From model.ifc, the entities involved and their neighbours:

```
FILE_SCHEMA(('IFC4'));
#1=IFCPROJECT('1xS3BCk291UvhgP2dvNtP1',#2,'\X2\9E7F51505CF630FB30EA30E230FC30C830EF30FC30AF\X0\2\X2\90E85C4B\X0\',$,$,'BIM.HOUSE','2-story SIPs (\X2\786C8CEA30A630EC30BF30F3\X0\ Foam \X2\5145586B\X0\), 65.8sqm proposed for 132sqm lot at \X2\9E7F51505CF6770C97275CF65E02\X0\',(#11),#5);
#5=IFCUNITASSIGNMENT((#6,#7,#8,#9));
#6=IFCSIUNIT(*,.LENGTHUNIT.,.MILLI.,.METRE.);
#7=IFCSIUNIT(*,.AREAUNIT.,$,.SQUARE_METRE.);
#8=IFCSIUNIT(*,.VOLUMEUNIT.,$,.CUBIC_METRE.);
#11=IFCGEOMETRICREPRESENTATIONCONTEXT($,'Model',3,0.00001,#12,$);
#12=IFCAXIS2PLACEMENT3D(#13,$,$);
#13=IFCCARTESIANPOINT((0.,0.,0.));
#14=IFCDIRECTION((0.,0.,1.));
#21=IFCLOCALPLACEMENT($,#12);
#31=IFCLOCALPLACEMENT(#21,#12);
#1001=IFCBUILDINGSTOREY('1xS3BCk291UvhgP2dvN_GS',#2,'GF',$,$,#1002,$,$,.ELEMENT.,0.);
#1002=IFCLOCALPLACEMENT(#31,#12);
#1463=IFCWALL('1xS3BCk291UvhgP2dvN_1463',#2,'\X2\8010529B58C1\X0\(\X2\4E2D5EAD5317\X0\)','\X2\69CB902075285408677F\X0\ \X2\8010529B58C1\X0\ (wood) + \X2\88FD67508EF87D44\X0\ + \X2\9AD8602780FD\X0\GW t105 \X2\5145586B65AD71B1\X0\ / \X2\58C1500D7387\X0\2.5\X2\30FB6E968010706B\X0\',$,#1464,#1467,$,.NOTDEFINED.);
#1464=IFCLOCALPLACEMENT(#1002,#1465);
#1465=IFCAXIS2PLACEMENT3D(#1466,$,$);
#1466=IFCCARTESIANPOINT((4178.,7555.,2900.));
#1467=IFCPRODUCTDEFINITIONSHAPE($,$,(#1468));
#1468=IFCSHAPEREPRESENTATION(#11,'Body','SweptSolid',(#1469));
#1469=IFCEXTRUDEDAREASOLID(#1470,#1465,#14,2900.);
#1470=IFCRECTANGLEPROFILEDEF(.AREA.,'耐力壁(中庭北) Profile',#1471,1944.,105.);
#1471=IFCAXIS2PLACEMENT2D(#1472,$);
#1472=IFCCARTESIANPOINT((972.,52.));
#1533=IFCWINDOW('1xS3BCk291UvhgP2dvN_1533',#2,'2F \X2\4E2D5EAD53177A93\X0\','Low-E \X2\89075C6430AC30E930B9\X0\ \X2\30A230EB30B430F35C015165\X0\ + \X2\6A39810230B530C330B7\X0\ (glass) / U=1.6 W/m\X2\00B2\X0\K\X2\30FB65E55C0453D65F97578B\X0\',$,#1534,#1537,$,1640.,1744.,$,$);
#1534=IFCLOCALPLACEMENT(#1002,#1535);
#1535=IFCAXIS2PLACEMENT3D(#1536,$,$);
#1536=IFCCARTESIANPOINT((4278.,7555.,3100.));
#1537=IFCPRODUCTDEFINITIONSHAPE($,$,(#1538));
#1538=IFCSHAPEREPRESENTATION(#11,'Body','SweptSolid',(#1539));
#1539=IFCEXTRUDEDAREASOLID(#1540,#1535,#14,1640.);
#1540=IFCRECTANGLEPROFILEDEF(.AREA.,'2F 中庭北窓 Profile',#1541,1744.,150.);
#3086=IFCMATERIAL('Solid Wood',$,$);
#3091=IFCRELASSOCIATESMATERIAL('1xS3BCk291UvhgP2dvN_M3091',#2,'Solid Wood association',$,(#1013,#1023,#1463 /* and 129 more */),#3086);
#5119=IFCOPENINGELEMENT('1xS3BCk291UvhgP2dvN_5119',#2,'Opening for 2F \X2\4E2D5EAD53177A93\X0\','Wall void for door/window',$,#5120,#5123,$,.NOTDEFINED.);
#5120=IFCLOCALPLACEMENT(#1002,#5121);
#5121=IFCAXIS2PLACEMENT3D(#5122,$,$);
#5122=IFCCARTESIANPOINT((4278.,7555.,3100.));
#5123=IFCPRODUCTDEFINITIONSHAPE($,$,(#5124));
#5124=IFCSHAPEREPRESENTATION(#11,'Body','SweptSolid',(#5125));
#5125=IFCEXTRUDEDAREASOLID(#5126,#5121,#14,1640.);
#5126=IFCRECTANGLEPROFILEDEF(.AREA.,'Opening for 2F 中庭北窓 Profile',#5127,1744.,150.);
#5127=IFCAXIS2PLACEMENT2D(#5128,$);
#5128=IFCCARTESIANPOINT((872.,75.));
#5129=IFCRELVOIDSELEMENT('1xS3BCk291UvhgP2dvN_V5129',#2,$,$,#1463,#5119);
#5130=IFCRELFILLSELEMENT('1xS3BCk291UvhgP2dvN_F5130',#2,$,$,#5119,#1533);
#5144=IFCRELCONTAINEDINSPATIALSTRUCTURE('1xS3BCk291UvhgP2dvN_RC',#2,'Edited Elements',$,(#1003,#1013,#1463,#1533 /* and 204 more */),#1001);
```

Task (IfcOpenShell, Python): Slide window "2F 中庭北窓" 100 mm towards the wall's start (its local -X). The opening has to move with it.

```python
import ifcopenshell
import ifcopenshell.api.geometry
import ifcopenshell.util.placement
import ifcopenshell.util.unit

model = ifcopenshell.open("model.ifc")
unit_scale = ifcopenshell.util.unit.calculate_unit_scale(model)

window = model.by_id(1533)
opening = window.FillsVoids[0].RelatingOpeningElement
wall = opening.VoidsElements[0].RelatingBuildingElement

wall_matrix = ifcopenshell.util.placement.get_local_placement(wall.ObjectPlacement)
shift = wall_matrix[:3, 0] * -0.1 / unit_scale
before = ifcopenshell.util.placement.get_local_placement(window.ObjectPlacement)[:3, 3].copy()

# The window is not placed relative to its opening, so move both.
for product in (opening, window):
    matrix = ifcopenshell.util.placement.get_local_placement(product.ObjectPlacement)
    matrix[:3, 3] += shift
    ifcopenshell.api.geometry.edit_object_placement(model, product=product, matrix=matrix, is_si=False)

after = ifcopenshell.util.placement.get_local_placement(window.ObjectPlacement)[:3, 3]
print("window moved by", (after - before).round(3) + 0.0)

model.write("model_updated.ifc")
```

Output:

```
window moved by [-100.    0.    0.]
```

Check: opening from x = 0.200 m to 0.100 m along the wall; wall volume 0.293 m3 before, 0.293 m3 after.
